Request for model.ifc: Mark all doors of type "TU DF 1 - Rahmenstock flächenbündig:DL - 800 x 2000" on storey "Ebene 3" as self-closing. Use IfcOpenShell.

First a look at what the model holds.

```python
import ifcopenshell
import ifcopenshell.util.element

model = ifcopenshell.open("model.ifc")
print(model.schema)
storey = next(s for s in model.by_type("IfcBuildingStorey") if s.Name == "Ebene 3")
doors = [e for e in ifcopenshell.util.element.get_decomposition(storey) if e.is_a("IfcDoor")]
seen = {}
for e in doors:
    element_type = ifcopenshell.util.element.get_type(e)
    key = (element_type.Name if element_type != e and element_type else None, ifcopenshell.util.element.get_pset(e, "Pset_DoorCommon", "SelfClosing"))
    seen[key] = seen.get(key, 0) + 1
for (name, value), count in sorted(seen.items(), key=str):
    print(count, "x", name, "|", value)
```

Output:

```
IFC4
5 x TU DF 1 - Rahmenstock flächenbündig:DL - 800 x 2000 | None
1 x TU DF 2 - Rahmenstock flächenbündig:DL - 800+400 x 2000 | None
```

```python
import ifcopenshell
import ifcopenshell.api.pset
import ifcopenshell.util.element

model = ifcopenshell.open("model.ifc")

storey = next(s for s in model.by_type("IfcBuildingStorey") if s.Name == "Ebene 3")
doors = [e for e in ifcopenshell.util.element.get_decomposition(storey) if e.is_a("IfcDoor")]

count = 0
for e in doors:
    element_type = ifcopenshell.util.element.get_type(e)
    if element_type in (None, e) or element_type.Name != "TU DF 1 - Rahmenstock flächenbündig:DL - 800 x 2000":
        continue
    # add_pset returns the element's existing set when there is one.
    pset = ifcopenshell.api.pset.add_pset(model, product=e, name="Pset_DoorCommon")
    ifcopenshell.api.pset.edit_pset(model, pset=pset, properties={"SelfClosing": True})
    count += 1

print(count, "doors updated")

model.write("model_edited.ifc")
```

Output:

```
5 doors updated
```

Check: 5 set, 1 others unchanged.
